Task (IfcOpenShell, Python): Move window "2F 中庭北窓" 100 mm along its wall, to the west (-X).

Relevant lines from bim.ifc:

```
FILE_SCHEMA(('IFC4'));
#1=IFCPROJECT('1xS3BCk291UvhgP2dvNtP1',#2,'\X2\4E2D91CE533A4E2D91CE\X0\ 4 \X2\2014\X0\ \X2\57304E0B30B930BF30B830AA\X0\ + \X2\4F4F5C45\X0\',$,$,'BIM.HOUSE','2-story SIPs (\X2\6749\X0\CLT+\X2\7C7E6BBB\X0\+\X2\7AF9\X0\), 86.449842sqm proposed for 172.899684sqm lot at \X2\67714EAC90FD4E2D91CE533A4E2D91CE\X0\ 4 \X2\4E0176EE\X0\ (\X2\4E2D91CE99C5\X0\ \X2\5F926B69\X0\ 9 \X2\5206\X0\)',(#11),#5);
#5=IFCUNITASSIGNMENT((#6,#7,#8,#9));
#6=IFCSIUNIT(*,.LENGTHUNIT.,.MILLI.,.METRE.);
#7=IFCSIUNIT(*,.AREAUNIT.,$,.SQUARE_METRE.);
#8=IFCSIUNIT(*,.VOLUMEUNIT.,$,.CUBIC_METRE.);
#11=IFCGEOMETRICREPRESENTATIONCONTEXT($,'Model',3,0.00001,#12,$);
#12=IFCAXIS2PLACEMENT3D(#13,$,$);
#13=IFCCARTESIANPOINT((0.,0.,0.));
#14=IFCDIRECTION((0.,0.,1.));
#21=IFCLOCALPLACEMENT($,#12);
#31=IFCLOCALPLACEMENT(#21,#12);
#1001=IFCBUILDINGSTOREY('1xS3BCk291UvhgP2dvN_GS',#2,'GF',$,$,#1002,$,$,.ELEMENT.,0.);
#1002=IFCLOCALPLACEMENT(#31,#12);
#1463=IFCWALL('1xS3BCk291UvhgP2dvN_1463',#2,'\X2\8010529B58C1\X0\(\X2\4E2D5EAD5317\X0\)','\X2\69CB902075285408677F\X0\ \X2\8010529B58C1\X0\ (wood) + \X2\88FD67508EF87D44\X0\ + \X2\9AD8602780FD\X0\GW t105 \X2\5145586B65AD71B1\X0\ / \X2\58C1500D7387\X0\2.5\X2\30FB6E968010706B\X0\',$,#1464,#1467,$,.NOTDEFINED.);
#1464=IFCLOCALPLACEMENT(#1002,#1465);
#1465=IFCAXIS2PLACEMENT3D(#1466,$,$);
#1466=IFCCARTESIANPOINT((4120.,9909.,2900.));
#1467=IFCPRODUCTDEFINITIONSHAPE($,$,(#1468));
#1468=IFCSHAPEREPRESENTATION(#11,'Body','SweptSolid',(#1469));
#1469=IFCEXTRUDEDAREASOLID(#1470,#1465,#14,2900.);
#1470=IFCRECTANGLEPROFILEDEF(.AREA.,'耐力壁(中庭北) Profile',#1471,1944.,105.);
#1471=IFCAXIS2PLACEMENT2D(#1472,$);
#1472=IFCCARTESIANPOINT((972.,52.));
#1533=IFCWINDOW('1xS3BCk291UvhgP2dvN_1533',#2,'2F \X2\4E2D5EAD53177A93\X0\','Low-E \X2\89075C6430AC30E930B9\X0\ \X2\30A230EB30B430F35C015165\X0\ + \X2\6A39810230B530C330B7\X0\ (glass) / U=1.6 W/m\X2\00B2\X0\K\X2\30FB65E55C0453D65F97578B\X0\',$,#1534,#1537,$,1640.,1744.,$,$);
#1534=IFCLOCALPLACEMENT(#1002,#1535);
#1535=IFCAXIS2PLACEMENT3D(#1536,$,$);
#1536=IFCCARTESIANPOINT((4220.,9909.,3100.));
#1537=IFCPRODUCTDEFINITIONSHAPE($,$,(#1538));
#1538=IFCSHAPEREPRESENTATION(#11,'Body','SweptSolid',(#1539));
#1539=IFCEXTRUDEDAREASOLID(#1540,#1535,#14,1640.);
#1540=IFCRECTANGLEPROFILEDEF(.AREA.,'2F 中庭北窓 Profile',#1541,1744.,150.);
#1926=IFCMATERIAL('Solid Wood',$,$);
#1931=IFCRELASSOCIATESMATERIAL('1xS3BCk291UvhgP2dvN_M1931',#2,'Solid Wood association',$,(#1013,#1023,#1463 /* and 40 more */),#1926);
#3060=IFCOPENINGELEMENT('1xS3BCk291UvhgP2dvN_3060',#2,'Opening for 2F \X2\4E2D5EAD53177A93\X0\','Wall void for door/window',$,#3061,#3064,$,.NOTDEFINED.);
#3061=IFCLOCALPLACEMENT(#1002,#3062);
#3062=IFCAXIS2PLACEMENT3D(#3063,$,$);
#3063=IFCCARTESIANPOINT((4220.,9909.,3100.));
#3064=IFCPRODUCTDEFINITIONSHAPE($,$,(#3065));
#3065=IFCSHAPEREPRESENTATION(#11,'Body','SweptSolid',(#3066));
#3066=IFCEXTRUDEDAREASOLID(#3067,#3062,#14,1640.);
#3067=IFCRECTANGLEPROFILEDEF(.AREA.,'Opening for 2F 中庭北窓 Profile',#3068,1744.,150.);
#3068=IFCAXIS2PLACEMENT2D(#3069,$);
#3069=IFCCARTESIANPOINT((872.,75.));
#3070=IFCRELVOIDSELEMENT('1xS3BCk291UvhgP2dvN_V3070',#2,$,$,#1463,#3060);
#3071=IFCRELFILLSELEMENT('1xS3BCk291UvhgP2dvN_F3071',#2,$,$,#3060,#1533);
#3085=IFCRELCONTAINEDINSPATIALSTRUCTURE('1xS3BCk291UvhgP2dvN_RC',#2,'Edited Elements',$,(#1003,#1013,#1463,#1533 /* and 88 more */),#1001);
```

```python
import ifcopenshell
import ifcopenshell.api.geometry
import ifcopenshell.util.placement

model = ifcopenshell.open("bim.ifc")

window = model.by_guid("1xS3BCk291UvhgP2dvN_1533")
opening = window.FillsVoids[0].RelatingOpeningElement
wall = opening.VoidsElements[0].RelatingBuildingElement

wall_matrix = ifcopenshell.util.placement.get_local_placement(wall.ObjectPlacement)
shift = wall_matrix[:3, 0] * -100.0
before = ifcopenshell.util.placement.get_local_placement(window.ObjectPlacement)[:3, 3].copy()

# The window is not placed relative to its opening, so move both.
for product in (opening, window):
    matrix = ifcopenshell.util.placement.get_local_placement(product.ObjectPlacement)
    matrix[:3, 3] += shift
    ifcopenshell.api.geometry.edit_object_placement(model, product=product, matrix=matrix, is_si=False)

after = ifcopenshell.util.placement.get_local_placement(window.ObjectPlacement)[:3, 3]
print("window moved by", (after - before).round(3) + 0.0)

model.write("bim-out.ifc")
```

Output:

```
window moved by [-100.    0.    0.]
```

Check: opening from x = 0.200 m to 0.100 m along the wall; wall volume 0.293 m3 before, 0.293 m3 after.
